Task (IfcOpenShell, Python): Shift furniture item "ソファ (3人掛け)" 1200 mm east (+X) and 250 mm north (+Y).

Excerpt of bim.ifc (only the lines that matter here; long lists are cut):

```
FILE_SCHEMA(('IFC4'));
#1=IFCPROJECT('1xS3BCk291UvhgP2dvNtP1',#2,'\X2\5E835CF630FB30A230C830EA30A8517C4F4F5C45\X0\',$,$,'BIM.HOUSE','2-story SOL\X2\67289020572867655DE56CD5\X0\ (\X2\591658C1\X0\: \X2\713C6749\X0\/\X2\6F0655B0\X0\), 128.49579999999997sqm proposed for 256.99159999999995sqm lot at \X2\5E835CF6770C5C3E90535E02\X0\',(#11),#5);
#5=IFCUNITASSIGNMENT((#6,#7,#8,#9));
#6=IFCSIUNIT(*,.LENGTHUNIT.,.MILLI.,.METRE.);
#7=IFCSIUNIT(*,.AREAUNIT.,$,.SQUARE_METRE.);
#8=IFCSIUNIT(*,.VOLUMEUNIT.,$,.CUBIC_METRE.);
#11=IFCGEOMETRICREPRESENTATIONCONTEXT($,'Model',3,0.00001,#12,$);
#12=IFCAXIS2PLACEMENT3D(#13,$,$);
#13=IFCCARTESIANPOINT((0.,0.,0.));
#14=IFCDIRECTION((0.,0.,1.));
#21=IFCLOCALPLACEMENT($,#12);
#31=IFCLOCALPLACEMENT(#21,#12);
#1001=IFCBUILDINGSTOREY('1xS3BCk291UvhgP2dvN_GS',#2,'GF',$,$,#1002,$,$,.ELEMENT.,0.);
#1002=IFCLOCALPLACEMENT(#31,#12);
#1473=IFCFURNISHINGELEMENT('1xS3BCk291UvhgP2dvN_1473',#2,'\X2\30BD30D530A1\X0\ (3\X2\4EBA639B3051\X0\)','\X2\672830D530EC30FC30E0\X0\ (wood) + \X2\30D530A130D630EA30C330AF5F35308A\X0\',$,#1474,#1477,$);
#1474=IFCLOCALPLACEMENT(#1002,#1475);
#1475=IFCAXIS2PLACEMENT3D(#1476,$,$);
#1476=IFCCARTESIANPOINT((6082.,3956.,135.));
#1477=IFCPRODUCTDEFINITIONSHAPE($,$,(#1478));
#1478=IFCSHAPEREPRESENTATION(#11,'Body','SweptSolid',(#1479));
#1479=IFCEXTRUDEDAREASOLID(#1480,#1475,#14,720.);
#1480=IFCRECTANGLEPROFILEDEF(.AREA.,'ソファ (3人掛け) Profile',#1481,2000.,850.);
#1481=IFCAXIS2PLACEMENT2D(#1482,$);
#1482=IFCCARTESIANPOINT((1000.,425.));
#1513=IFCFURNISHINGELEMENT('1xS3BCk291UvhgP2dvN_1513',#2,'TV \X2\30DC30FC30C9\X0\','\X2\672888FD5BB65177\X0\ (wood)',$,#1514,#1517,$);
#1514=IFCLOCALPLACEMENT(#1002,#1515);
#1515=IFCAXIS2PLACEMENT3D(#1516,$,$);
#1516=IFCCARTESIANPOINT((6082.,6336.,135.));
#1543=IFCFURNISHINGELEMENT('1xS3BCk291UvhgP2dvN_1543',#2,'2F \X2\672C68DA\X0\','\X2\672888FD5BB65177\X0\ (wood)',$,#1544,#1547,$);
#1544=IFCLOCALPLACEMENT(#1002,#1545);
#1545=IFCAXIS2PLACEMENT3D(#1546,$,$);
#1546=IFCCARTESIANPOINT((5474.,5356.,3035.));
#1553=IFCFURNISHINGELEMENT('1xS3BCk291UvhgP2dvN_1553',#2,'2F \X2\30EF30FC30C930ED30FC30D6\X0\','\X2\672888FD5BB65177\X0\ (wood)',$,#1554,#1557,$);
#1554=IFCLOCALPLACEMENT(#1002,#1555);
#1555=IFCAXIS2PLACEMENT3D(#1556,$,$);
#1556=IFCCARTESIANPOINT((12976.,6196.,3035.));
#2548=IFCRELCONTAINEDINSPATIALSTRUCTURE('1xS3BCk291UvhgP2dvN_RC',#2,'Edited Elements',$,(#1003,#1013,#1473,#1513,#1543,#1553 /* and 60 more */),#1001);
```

```python
import ifcopenshell
import ifcopenshell.api.geometry
import ifcopenshell.util.placement
import ifcopenshell.util.unit

model = ifcopenshell.open("bim.ifc")
unit_scale = ifcopenshell.util.unit.calculate_unit_scale(model)

item = model.by_guid("1xS3BCk291UvhgP2dvN_1473")
matrix = ifcopenshell.util.placement.get_local_placement(item.ObjectPlacement)
matrix[0, 3] += 1.2 / unit_scale
matrix[1, 3] += 0.25 / unit_scale
ifcopenshell.api.geometry.edit_object_placement(model, product=item, matrix=matrix, is_si=False)

print(ifcopenshell.util.placement.get_local_placement(item.ObjectPlacement).round(3) + 0.0)

model.write("bim_rev.ifc")
```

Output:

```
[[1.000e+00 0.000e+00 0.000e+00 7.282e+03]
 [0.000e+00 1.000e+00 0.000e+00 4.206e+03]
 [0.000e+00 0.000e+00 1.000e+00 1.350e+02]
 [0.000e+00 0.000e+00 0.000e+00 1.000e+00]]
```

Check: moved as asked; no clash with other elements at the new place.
